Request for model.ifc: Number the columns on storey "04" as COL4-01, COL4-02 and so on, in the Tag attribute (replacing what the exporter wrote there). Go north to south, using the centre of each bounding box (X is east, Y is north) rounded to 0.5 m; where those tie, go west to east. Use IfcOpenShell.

First a look at what the model holds.

```python
import ifcopenshell
import ifcopenshell.util.element
import ifcopenshell.util.placement

model = ifcopenshell.open("model.ifc")
print(model.schema)
storey = next(s for s in model.by_type("IfcBuildingStorey") if s.Name == "04")
columns = [e for e in ifcopenshell.util.element.get_decomposition(storey) if e.is_a("IfcColumn")]
for e in sorted(columns, key=lambda e: e.id()):
    origin = ifcopenshell.util.placement.get_local_placement(e.ObjectPlacement)[:3, 3]
    print(e.id(), e.Tag, e.Name, origin.round(2) + 0.0, sep=" | ")
```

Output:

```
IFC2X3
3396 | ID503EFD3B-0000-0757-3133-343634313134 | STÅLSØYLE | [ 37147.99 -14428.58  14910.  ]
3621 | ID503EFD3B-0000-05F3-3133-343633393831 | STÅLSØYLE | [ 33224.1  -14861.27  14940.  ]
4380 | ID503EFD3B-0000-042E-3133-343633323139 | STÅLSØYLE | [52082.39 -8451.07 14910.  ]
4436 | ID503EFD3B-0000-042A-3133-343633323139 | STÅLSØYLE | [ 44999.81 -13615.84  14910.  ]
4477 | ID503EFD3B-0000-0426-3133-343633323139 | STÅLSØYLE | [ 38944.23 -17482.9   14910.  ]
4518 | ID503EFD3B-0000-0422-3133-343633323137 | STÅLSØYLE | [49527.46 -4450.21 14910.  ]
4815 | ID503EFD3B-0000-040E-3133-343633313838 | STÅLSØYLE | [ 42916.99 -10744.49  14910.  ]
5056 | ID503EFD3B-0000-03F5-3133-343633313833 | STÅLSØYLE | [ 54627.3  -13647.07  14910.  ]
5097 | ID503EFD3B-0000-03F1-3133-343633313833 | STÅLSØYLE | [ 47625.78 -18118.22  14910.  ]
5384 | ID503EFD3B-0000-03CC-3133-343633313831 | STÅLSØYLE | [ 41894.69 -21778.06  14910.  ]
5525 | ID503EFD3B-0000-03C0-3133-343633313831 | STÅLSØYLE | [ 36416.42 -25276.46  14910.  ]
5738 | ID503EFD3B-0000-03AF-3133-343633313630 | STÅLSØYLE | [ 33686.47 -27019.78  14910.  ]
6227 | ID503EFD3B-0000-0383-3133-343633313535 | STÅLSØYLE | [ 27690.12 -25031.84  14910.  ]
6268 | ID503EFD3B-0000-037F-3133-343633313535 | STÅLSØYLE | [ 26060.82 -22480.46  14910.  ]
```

```python
import ifcopenshell
import ifcopenshell.geom
import ifcopenshell.util.element
import ifcopenshell.util.shape

model = ifcopenshell.open("model.ifc")
settings = ifcopenshell.geom.settings()
settings.set("use-world-coords", True)


def centre(element):
    shape = ifcopenshell.geom.create_shape(settings, element)
    return ifcopenshell.util.shape.get_bbox_centroid(shape.geometry)


storey = next(s for s in model.by_type("IfcBuildingStorey") if s.Name == "04")
columns = [e for e in ifcopenshell.util.element.get_decomposition(storey) if e.is_a("IfcColumn")]

# Insertion points can sit at a corner or the storey origin, so sort by the geometry (in metres).
centres = {e: centre(e) for e in columns}
columns.sort(key=lambda e: (-round(centres[e][1] / 0.5), centres[e][0]))

for i, e in enumerate(columns, start=1):
    number = f"COL4-{i:02d}"
    e.Tag = number
    print(e.id(), number)

model.write("model_updated.ifc")
```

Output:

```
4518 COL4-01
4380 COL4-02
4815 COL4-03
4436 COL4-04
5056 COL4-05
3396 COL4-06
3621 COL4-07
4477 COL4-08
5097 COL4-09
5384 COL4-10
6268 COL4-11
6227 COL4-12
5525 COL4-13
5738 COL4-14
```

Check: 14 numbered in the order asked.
